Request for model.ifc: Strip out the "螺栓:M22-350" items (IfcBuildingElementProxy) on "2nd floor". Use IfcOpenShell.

First a look at what the model holds.

```python
import ifcopenshell
import ifcopenshell.util.element

model = ifcopenshell.open("model.ifc")
print(model.schema)
storey = next(s for s in model.by_type("IfcBuildingStorey") if s.Name == "2nd floor")
proxies = [e for e in ifcopenshell.util.element.get_decomposition(storey) if e.is_a("IfcBuildingElementProxy")]
seen = {}
for e in proxies:
    element_type = ifcopenshell.util.element.get_type(e)
    name = element_type.Name if element_type not in (None, e) else None
    seen[name] = seen.get(name, 0) + 1
for name, count in sorted(seen.items(), key=str):
    print(count, "x", name)
```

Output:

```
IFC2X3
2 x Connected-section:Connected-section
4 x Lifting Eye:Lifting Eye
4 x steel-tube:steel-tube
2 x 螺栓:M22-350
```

```python
import ifcopenshell
import ifcopenshell.api.root
import ifcopenshell.util.element

model = ifcopenshell.open("model.ifc")

storey = next(s for s in model.by_type("IfcBuildingStorey") if s.Name == "2nd floor")
proxies = [e for e in ifcopenshell.util.element.get_decomposition(storey) if e.is_a("IfcBuildingElementProxy")]
targets = [e for e in proxies if (t := ifcopenshell.util.element.get_type(e)) not in (None, e) and t.Name == "螺栓:M22-350"]

for e in targets:
    ifcopenshell.api.root.remove_product(model, product=e)
print(len(targets), "removed")

model.write("model-out.ifc")
```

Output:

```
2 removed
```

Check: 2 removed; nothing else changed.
